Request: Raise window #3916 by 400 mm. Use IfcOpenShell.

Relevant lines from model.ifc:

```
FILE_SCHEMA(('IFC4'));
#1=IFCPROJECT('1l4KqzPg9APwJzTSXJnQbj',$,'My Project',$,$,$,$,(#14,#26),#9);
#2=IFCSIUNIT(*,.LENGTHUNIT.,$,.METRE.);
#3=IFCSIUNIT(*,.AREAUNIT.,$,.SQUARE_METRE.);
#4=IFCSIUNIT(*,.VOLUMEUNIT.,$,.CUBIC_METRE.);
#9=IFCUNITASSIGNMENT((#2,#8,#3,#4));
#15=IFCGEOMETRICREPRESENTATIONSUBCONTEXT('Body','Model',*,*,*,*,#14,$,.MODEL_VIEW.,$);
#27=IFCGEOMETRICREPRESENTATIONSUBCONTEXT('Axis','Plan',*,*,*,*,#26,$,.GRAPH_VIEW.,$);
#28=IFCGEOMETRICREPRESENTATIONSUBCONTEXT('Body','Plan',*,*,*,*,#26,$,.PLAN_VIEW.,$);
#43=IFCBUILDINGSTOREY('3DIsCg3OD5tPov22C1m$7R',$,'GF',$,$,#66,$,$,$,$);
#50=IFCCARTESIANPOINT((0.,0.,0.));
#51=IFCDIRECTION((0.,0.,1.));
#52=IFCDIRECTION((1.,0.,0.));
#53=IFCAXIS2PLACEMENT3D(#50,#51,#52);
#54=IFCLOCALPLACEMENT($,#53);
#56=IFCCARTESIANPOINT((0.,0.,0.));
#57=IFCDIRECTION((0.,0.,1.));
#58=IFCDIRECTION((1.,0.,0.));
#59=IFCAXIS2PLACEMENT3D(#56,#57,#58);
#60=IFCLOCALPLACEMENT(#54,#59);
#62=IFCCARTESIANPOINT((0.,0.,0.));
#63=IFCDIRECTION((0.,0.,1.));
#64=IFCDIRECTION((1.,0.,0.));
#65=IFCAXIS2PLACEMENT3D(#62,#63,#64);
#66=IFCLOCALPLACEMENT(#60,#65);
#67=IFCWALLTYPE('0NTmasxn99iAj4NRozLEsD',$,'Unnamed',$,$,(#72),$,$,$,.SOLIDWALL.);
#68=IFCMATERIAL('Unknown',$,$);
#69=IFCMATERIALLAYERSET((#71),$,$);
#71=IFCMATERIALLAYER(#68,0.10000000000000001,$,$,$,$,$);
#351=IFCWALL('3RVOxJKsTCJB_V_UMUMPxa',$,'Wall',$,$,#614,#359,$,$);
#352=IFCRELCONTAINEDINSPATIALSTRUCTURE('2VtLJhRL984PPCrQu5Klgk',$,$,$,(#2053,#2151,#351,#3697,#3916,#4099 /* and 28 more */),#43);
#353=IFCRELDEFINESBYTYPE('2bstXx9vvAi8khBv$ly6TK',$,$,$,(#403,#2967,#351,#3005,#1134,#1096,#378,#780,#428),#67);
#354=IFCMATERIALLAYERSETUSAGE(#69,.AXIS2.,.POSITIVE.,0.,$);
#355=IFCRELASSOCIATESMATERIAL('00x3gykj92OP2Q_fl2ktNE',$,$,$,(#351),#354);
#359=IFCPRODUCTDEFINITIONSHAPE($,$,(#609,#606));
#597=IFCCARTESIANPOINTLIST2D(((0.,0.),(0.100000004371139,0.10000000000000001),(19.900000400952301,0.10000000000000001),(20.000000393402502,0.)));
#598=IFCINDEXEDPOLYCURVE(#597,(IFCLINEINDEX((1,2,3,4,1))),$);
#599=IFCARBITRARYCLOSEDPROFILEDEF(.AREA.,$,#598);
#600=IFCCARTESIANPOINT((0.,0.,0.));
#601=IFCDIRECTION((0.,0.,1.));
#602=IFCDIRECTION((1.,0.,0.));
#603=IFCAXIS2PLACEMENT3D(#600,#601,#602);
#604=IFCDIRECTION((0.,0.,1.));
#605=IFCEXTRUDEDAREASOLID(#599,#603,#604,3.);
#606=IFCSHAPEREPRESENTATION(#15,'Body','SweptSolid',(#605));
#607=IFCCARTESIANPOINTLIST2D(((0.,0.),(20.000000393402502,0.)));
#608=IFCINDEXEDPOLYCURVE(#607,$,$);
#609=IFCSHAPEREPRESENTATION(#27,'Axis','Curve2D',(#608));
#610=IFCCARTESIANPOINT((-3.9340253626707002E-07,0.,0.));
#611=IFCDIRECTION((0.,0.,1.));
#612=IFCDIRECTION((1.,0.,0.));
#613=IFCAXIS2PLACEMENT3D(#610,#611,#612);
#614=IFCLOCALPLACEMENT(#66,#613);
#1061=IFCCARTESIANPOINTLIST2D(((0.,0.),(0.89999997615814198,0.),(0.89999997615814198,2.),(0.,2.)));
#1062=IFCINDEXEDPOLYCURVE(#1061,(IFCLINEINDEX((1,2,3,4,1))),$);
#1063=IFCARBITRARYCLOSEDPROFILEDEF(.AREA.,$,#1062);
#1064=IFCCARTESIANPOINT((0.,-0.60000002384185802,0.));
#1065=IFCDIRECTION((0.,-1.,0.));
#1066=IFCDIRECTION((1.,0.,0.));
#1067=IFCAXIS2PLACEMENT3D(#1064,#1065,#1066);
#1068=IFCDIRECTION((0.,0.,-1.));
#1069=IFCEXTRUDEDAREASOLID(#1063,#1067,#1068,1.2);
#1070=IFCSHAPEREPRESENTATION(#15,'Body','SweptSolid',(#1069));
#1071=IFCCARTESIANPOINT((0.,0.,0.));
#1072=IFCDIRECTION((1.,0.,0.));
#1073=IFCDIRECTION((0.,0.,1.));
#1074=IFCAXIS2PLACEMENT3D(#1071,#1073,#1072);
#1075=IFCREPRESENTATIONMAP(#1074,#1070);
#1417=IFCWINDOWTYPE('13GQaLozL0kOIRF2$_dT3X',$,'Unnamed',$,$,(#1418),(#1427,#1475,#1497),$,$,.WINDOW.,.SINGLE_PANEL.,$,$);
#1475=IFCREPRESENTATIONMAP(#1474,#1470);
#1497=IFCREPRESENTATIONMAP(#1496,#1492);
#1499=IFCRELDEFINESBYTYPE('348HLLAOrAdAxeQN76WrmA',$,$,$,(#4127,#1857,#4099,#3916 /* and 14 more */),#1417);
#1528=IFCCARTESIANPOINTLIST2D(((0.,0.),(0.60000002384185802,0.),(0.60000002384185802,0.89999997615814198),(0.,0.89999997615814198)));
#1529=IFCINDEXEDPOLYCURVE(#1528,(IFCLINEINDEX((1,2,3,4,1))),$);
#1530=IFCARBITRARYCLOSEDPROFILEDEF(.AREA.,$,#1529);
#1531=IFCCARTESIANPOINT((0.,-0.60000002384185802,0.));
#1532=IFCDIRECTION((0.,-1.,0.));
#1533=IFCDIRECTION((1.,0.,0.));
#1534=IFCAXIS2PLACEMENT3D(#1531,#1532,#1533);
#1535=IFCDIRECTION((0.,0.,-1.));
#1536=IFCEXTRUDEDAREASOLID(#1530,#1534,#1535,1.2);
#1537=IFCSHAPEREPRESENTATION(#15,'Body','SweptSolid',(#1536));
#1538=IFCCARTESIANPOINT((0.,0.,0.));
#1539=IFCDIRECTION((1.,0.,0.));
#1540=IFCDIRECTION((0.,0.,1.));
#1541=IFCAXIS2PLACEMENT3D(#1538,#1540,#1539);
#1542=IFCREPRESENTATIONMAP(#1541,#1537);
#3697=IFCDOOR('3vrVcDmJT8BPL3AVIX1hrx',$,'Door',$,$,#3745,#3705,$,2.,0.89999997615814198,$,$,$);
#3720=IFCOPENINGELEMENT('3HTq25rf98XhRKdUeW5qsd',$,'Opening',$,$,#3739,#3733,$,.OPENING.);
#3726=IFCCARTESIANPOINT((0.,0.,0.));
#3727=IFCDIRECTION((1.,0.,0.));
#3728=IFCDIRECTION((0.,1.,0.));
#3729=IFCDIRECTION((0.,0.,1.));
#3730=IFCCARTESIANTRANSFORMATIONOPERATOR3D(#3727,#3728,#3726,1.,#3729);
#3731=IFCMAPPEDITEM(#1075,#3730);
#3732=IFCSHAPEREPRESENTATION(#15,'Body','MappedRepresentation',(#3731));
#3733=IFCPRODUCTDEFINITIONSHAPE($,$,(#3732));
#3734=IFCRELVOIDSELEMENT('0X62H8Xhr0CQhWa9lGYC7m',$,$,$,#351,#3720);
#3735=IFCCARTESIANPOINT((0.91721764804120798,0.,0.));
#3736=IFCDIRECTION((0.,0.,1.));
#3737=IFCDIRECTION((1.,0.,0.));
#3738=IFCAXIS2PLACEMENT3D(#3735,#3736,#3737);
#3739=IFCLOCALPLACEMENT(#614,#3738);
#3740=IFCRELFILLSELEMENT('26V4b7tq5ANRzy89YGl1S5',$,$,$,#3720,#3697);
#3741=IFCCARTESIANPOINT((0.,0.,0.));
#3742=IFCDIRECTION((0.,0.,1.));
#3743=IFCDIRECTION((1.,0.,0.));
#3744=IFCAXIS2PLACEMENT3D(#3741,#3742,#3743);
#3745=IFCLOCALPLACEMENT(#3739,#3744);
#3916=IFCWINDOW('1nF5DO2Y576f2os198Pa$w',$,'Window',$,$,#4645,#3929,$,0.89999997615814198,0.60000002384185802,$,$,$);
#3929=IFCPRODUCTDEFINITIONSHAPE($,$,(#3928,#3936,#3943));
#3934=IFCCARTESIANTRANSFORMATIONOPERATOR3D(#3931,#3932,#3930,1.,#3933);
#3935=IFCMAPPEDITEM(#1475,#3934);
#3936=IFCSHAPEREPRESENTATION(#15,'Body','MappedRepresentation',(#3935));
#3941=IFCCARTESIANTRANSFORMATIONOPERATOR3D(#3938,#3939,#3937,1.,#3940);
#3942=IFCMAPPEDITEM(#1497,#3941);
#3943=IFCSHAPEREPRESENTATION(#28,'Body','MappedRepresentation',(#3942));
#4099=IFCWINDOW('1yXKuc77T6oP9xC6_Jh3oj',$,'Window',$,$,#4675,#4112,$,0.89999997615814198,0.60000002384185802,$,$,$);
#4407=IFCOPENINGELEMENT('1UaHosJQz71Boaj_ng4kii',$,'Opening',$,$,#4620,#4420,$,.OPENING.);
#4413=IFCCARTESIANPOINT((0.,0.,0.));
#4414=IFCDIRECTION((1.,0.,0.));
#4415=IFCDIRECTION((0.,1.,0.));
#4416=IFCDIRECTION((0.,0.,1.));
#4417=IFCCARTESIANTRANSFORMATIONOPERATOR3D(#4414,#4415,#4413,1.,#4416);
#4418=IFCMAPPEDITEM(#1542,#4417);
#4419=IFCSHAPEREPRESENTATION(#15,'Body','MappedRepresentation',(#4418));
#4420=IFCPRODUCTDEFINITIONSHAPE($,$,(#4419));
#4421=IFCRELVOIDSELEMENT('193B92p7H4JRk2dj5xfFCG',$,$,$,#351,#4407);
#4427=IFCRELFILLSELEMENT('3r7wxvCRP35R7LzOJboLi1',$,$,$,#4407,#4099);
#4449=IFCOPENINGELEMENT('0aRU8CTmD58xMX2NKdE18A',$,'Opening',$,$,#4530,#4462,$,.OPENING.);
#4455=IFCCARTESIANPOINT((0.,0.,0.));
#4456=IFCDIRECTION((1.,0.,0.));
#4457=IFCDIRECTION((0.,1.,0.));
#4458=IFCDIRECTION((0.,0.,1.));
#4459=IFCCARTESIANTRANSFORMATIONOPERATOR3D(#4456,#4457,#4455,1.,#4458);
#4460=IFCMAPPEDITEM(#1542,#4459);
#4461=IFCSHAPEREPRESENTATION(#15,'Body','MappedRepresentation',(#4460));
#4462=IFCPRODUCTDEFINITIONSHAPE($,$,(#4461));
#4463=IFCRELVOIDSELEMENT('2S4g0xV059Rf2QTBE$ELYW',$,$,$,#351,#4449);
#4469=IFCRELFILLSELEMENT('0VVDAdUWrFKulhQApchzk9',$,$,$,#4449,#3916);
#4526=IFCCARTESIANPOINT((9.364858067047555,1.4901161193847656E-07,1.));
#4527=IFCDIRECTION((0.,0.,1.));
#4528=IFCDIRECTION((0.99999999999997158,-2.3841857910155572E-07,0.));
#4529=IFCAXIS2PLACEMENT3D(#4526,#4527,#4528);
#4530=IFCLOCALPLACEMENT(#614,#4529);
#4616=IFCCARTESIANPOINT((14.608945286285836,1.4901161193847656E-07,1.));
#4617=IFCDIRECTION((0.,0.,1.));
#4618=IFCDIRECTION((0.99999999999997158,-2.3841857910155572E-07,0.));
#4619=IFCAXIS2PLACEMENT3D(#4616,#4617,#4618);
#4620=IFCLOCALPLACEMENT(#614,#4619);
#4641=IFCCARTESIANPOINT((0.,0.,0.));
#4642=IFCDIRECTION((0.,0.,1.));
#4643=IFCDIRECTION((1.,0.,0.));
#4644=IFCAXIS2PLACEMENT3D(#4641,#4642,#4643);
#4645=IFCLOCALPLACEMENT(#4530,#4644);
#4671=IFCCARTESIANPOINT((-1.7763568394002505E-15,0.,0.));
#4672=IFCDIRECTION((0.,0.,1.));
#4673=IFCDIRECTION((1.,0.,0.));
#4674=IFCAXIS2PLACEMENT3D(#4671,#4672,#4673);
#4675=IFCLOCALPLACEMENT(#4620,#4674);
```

```python
import numpy as np
import ifcopenshell
import ifcopenshell.api.geometry
import ifcopenshell.util.placement
import ifcopenshell.util.unit

model = ifcopenshell.open("model.ifc")
unit_scale = ifcopenshell.util.unit.calculate_unit_scale(model)

window = model.by_guid("1nF5DO2Y576f2os198Pa$w")
opening = window.FillsVoids[0].RelatingOpeningElement
dz = 0.4 / unit_scale

shift = np.array([0.0, 0.0, dz])
# The window is placed relative to its opening, so it follows when the opening moves.
matrix = ifcopenshell.util.placement.get_local_placement(opening.ObjectPlacement)
matrix[:3, 3] += shift
ifcopenshell.api.geometry.edit_object_placement(
    model, product=opening, matrix=matrix, is_si=False, should_transform_children=True
)

print(f"moved by {dz * unit_scale:+.3f} m")

model.write("model_updated.ifc")
```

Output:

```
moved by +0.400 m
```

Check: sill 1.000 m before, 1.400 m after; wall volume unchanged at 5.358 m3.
